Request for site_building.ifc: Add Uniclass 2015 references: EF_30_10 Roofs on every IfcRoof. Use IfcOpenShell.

First a look at what the model holds.

```python
import ifcopenshell

model = ifcopenshell.open("site_building.ifc")
print(model.schema)
print("classifications:", [c.Name for c in model.by_type("IfcClassification")])
for ifc_class in ("IfcDoor", "IfcRoof", "IfcStair", "IfcWall", "IfcWindow"):
    print(ifc_class, len(model.by_type(ifc_class)))
```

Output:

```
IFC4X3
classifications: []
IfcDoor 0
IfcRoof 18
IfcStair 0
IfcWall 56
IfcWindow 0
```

```python
import ifcopenshell
import ifcopenshell.api.classification

model = ifcopenshell.open("site_building.ifc")

system = ifcopenshell.api.classification.add_classification(model, classification="Uniclass 2015")

codes = {
    "IfcRoof": ("EF_30_10", "Roofs"),
}
for ifc_class, (code, name) in codes.items():
    products = model.by_type(ifc_class)
    ifcopenshell.api.classification.add_reference(
        model, products=products, classification=system, identification=code, name=name
    )
    print(code, len(products))

model.write("site_building_rev.ifc")
```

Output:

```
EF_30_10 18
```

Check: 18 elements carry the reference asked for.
